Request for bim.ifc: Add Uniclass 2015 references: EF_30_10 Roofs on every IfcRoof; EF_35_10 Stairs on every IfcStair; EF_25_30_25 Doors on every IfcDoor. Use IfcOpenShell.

First a look at what the model holds.

```python
import ifcopenshell

model = ifcopenshell.open("bim.ifc")
print(model.schema)
print("classifications:", [c.Name for c in model.by_type("IfcClassification")])
for ifc_class in ("IfcDoor", "IfcRoof", "IfcStair", "IfcWall", "IfcWindow"):
    print(ifc_class, len(model.by_type(ifc_class)))
```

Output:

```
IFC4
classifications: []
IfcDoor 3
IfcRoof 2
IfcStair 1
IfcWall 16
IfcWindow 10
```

```python
import ifcopenshell
import ifcopenshell.api.classification

model = ifcopenshell.open("bim.ifc")

system = ifcopenshell.api.classification.add_classification(model, classification="Uniclass 2015")

codes = {
    "IfcRoof": ("EF_30_10", "Roofs"),
    "IfcStair": ("EF_35_10", "Stairs"),
    "IfcDoor": ("EF_25_30_25", "Doors"),
}
for ifc_class, (code, name) in codes.items():
    products = model.by_type(ifc_class)
    ifcopenshell.api.classification.add_reference(
        model, products=products, classification=system, identification=code, name=name
    )
    print(code, len(products))

model.write("bim_edited.ifc")
```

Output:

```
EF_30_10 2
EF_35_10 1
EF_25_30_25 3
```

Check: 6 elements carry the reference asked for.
